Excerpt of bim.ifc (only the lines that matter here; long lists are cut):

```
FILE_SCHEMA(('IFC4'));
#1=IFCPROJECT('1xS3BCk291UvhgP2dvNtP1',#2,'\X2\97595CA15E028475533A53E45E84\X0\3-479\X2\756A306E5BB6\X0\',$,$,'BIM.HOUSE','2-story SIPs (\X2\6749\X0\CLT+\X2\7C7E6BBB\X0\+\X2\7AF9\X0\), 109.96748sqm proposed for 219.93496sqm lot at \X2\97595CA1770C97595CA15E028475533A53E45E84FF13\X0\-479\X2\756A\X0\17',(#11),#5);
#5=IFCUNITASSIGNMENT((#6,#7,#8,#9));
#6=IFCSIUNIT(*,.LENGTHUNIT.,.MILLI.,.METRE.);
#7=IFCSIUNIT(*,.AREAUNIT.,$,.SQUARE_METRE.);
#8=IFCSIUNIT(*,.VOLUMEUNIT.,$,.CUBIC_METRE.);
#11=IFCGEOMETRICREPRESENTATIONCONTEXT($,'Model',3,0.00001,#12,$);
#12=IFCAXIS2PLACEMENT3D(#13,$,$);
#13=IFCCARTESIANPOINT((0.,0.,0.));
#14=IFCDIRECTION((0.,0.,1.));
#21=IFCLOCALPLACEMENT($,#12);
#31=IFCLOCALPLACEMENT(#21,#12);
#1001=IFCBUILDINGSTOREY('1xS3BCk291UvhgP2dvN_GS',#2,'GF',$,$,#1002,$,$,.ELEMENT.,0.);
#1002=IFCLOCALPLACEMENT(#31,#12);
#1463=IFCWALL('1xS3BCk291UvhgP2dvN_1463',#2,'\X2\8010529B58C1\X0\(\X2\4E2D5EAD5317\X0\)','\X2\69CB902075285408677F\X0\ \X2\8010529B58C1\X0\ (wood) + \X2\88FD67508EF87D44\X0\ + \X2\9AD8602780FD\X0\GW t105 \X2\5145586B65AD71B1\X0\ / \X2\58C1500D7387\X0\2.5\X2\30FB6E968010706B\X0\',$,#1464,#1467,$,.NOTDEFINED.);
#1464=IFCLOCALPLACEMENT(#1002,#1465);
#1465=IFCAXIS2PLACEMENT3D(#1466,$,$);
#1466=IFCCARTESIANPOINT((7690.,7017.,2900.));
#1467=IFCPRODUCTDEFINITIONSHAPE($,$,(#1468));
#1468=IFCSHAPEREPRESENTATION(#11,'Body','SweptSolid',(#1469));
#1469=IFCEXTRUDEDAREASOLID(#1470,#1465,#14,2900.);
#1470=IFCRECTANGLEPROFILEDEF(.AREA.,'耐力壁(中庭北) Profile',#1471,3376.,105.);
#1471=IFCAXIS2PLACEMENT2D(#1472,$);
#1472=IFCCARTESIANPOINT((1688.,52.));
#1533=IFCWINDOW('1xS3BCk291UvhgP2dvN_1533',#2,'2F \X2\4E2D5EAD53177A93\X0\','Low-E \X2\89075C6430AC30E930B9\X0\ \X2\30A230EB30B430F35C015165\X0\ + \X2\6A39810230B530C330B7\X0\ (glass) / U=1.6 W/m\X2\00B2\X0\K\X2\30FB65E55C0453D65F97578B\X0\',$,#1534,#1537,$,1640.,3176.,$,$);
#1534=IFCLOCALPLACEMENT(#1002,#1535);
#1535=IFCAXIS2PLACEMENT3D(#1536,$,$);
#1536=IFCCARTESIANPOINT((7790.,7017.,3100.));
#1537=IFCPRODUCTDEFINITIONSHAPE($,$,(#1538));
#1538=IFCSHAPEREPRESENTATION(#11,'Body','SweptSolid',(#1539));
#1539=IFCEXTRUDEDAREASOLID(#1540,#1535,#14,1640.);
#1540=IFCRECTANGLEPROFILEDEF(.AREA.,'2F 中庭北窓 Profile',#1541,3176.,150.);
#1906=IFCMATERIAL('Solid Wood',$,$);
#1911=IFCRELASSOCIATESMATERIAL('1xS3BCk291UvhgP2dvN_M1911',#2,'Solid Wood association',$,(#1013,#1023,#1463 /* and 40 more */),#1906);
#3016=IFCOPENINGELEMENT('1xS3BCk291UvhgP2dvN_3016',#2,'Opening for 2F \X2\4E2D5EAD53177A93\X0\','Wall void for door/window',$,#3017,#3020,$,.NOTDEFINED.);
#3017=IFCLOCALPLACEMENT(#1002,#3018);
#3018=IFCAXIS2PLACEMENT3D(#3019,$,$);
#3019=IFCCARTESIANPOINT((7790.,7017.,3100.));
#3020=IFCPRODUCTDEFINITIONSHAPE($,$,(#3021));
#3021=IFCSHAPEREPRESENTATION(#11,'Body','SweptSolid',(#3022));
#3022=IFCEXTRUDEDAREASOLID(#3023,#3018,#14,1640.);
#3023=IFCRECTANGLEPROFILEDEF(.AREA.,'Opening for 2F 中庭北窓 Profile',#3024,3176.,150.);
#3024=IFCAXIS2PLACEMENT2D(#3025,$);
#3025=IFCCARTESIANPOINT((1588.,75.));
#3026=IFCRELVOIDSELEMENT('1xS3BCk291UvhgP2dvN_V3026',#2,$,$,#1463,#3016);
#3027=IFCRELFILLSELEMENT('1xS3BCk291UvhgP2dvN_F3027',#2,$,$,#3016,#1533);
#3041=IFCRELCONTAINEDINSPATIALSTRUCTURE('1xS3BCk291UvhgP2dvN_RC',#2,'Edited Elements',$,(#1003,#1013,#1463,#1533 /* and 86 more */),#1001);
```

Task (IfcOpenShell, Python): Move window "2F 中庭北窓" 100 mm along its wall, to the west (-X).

```python
import ifcopenshell
import ifcopenshell.api.geometry
import ifcopenshell.util.placement
import ifcopenshell.util.unit

model = ifcopenshell.open("bim.ifc")
unit_scale = ifcopenshell.util.unit.calculate_unit_scale(model)

window = model.by_guid("1xS3BCk291UvhgP2dvN_1533")
opening = window.FillsVoids[0].RelatingOpeningElement
wall = opening.VoidsElements[0].RelatingBuildingElement

wall_matrix = ifcopenshell.util.placement.get_local_placement(wall.ObjectPlacement)
shift = wall_matrix[:3, 0] * -0.1 / unit_scale
before = ifcopenshell.util.placement.get_local_placement(window.ObjectPlacement)[:3, 3].copy()

# The window is not placed relative to its opening, so move both.
for product in (opening, window):
    matrix = ifcopenshell.util.placement.get_local_placement(product.ObjectPlacement)
    matrix[:3, 3] += shift
    ifcopenshell.api.geometry.edit_object_placement(model, product=product, matrix=matrix, is_si=False)

after = ifcopenshell.util.placement.get_local_placement(window.ObjectPlacement)[:3, 3]
print("window moved by", (after - before).round(3) + 0.0)

model.write("bim-out.ifc")
```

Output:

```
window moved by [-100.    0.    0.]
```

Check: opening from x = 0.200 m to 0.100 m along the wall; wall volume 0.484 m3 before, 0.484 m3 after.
